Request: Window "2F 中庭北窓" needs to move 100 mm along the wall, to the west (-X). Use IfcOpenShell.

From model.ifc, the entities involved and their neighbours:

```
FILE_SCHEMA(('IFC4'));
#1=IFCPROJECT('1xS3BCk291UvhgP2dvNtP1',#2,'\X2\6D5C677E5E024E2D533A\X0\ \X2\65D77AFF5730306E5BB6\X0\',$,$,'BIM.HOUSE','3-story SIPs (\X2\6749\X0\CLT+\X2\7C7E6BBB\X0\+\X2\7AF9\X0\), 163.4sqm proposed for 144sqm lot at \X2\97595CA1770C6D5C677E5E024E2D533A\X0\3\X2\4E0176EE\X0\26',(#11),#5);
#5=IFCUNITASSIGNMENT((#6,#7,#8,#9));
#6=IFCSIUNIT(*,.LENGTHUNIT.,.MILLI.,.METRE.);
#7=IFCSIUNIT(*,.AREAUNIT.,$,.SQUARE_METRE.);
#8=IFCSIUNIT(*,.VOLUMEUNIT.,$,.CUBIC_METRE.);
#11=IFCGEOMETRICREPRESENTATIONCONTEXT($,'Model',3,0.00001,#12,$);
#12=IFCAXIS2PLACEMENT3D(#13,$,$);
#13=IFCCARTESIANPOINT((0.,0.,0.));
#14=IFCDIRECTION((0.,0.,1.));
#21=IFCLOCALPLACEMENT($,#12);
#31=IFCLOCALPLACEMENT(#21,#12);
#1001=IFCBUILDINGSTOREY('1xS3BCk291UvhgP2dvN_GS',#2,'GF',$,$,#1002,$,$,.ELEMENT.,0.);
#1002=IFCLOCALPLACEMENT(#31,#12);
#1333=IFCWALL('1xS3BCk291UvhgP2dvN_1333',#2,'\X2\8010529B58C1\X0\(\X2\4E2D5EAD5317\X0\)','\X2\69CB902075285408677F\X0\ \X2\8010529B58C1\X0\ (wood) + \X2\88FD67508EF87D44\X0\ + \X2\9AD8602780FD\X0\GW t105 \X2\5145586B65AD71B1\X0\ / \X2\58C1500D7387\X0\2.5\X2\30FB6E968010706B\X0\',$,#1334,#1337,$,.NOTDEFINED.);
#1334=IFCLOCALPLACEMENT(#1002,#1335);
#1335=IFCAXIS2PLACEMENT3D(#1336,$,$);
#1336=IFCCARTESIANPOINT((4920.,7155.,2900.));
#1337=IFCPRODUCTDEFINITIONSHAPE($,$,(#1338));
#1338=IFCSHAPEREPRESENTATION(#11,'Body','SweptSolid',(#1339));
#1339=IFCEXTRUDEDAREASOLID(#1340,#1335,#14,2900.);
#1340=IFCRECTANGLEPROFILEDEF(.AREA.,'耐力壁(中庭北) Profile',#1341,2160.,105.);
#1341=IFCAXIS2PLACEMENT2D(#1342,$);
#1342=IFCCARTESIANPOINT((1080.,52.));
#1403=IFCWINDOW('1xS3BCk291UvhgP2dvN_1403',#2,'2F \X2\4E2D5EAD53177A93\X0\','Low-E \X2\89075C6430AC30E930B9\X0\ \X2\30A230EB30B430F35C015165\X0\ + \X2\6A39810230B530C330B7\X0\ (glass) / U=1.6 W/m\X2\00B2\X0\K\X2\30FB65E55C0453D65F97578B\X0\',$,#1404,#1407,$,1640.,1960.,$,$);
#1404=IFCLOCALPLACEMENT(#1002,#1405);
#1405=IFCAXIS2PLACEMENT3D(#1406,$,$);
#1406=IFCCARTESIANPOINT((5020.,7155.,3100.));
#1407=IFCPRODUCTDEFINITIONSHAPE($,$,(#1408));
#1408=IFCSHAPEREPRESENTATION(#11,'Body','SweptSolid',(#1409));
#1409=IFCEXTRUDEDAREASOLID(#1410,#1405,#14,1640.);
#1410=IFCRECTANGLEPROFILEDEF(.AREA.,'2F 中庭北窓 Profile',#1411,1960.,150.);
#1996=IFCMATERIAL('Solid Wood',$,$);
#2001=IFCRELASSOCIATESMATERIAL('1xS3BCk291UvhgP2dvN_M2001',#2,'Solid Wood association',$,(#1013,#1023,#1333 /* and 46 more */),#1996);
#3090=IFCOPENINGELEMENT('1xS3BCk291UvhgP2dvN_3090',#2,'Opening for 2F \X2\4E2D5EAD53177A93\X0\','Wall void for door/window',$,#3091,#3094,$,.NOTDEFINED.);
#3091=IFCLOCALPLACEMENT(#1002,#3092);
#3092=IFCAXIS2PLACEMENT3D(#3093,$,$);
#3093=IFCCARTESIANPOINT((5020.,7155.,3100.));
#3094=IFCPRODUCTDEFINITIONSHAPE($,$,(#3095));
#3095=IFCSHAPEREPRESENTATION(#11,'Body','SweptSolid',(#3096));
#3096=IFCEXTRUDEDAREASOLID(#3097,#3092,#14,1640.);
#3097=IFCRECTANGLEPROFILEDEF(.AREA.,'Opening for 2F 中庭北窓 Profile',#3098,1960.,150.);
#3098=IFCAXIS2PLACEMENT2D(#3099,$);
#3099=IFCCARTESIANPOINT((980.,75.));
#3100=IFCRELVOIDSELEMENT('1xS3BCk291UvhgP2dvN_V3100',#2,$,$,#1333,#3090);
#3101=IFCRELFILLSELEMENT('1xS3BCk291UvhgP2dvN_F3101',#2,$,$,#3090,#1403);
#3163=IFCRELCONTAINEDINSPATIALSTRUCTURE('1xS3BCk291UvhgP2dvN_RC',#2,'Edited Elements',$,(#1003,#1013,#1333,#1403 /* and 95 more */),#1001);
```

```python
import ifcopenshell
import ifcopenshell.api.geometry
import ifcopenshell.util.placement
import ifcopenshell.util.unit

model = ifcopenshell.open("model.ifc")
unit_scale = ifcopenshell.util.unit.calculate_unit_scale(model)

window = model.by_guid("1xS3BCk291UvhgP2dvN_1403")
opening = window.FillsVoids[0].RelatingOpeningElement
wall = opening.VoidsElements[0].RelatingBuildingElement

wall_matrix = ifcopenshell.util.placement.get_local_placement(wall.ObjectPlacement)
shift = wall_matrix[:3, 0] * -0.1 / unit_scale
before = ifcopenshell.util.placement.get_local_placement(window.ObjectPlacement)[:3, 3].copy()

# The window is not placed relative to its opening, so move both.
for product in (opening, window):
    matrix = ifcopenshell.util.placement.get_local_placement(product.ObjectPlacement)
    matrix[:3, 3] += shift
    ifcopenshell.api.geometry.edit_object_placement(model, product=product, matrix=matrix, is_si=False)

after = ifcopenshell.util.placement.get_local_placement(window.ObjectPlacement)[:3, 3]
print("window moved by", (after - before).round(3) + 0.0)

model.write("model_v2.ifc")
```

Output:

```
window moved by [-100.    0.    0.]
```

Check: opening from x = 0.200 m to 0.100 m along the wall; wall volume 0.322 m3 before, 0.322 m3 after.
